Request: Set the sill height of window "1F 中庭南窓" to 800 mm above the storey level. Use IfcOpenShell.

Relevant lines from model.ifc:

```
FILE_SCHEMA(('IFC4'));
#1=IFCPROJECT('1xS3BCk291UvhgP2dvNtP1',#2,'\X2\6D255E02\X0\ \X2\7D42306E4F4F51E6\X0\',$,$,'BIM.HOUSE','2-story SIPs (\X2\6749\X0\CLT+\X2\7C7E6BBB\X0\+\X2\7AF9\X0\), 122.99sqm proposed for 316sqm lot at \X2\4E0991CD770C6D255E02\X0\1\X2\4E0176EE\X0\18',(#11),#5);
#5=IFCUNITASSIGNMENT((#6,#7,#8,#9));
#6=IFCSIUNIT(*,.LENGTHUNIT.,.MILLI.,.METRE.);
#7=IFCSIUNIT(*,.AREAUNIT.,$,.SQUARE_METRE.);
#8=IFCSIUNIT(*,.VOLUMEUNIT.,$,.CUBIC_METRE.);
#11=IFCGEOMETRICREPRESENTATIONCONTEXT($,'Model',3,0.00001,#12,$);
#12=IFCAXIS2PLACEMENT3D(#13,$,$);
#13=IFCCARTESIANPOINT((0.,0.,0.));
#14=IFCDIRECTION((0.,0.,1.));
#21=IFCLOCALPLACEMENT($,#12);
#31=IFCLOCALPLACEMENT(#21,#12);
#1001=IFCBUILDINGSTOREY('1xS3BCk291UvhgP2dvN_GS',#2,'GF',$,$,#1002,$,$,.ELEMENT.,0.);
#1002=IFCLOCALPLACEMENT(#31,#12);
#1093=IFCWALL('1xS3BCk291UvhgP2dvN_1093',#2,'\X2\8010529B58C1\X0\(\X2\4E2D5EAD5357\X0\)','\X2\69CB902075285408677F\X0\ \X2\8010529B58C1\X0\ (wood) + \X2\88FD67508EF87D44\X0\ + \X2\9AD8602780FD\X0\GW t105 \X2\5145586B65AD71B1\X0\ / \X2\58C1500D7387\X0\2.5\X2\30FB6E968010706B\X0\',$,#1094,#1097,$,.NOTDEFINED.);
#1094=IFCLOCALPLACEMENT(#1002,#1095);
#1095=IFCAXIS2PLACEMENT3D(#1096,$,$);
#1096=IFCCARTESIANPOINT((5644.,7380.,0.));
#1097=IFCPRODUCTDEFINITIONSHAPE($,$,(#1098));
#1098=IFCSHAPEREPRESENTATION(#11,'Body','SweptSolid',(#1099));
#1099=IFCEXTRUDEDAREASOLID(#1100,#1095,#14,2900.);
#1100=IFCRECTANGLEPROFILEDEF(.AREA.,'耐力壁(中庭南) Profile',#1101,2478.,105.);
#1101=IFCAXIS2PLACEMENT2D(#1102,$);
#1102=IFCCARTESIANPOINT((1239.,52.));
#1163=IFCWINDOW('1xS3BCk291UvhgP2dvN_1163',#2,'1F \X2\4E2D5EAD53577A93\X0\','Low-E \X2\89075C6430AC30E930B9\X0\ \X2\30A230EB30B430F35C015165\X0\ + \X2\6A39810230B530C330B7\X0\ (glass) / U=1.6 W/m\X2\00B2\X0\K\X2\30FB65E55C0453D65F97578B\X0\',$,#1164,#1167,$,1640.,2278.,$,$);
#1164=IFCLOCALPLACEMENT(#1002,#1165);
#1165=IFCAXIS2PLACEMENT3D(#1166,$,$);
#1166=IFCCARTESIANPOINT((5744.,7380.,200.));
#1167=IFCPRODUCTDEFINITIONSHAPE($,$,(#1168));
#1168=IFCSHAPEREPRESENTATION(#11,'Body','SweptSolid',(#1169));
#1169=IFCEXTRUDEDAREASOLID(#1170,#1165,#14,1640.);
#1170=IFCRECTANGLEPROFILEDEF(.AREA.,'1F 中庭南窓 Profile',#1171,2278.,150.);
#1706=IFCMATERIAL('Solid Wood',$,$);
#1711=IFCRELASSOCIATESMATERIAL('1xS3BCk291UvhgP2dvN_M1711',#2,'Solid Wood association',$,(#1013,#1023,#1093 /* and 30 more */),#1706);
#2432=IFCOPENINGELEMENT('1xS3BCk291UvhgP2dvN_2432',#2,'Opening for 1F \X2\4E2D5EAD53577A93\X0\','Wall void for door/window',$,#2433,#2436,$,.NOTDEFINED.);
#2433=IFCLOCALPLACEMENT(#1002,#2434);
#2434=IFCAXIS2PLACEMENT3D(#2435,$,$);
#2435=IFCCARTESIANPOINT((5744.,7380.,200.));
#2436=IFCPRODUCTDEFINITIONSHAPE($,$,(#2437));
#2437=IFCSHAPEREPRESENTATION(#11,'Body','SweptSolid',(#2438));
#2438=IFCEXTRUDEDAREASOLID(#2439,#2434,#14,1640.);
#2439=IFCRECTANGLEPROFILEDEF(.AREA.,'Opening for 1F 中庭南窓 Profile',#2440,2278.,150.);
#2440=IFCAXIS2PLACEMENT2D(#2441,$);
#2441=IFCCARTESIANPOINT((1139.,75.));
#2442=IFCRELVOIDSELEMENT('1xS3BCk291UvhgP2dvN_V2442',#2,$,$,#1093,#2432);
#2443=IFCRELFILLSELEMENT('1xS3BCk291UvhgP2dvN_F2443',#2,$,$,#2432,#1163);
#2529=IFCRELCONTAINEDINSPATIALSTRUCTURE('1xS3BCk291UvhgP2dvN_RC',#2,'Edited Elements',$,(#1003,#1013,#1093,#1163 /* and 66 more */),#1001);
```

```python
import numpy as np
import ifcopenshell
import ifcopenshell.api.geometry
import ifcopenshell.geom
import ifcopenshell.util.element
import ifcopenshell.util.placement
import ifcopenshell.util.shape
import ifcopenshell.util.unit

model = ifcopenshell.open("model.ifc")
unit_scale = ifcopenshell.util.unit.calculate_unit_scale(model)

window = model.by_id(1163)
opening = window.FillsVoids[0].RelatingOpeningElement
storey = ifcopenshell.util.element.get_container(window, ifc_class="IfcBuildingStorey")
level = ifcopenshell.util.placement.get_local_placement(storey.ObjectPlacement)[2, 3]

# The opening's origin need not be at the sill, so measure its lowest point.
shape = ifcopenshell.geom.create_shape(ifcopenshell.geom.settings(), opening)
bottom = ifcopenshell.util.shape.get_shape_bottom_elevation(shape, shape.geometry) / unit_scale
dz = level + 800.0 - bottom

shift = np.array([0.0, 0.0, dz])
# The window is not placed relative to its opening, so move both.
for product in (opening, window):
    matrix = ifcopenshell.util.placement.get_local_placement(product.ObjectPlacement)
    matrix[:3, 3] += shift
    ifcopenshell.api.geometry.edit_object_placement(model, product=product, matrix=matrix, is_si=False)

print(f"moved by {dz * unit_scale:+.3f} m")

model.write("model_v2.ifc")
```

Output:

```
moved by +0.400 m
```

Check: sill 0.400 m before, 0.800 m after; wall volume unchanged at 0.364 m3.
